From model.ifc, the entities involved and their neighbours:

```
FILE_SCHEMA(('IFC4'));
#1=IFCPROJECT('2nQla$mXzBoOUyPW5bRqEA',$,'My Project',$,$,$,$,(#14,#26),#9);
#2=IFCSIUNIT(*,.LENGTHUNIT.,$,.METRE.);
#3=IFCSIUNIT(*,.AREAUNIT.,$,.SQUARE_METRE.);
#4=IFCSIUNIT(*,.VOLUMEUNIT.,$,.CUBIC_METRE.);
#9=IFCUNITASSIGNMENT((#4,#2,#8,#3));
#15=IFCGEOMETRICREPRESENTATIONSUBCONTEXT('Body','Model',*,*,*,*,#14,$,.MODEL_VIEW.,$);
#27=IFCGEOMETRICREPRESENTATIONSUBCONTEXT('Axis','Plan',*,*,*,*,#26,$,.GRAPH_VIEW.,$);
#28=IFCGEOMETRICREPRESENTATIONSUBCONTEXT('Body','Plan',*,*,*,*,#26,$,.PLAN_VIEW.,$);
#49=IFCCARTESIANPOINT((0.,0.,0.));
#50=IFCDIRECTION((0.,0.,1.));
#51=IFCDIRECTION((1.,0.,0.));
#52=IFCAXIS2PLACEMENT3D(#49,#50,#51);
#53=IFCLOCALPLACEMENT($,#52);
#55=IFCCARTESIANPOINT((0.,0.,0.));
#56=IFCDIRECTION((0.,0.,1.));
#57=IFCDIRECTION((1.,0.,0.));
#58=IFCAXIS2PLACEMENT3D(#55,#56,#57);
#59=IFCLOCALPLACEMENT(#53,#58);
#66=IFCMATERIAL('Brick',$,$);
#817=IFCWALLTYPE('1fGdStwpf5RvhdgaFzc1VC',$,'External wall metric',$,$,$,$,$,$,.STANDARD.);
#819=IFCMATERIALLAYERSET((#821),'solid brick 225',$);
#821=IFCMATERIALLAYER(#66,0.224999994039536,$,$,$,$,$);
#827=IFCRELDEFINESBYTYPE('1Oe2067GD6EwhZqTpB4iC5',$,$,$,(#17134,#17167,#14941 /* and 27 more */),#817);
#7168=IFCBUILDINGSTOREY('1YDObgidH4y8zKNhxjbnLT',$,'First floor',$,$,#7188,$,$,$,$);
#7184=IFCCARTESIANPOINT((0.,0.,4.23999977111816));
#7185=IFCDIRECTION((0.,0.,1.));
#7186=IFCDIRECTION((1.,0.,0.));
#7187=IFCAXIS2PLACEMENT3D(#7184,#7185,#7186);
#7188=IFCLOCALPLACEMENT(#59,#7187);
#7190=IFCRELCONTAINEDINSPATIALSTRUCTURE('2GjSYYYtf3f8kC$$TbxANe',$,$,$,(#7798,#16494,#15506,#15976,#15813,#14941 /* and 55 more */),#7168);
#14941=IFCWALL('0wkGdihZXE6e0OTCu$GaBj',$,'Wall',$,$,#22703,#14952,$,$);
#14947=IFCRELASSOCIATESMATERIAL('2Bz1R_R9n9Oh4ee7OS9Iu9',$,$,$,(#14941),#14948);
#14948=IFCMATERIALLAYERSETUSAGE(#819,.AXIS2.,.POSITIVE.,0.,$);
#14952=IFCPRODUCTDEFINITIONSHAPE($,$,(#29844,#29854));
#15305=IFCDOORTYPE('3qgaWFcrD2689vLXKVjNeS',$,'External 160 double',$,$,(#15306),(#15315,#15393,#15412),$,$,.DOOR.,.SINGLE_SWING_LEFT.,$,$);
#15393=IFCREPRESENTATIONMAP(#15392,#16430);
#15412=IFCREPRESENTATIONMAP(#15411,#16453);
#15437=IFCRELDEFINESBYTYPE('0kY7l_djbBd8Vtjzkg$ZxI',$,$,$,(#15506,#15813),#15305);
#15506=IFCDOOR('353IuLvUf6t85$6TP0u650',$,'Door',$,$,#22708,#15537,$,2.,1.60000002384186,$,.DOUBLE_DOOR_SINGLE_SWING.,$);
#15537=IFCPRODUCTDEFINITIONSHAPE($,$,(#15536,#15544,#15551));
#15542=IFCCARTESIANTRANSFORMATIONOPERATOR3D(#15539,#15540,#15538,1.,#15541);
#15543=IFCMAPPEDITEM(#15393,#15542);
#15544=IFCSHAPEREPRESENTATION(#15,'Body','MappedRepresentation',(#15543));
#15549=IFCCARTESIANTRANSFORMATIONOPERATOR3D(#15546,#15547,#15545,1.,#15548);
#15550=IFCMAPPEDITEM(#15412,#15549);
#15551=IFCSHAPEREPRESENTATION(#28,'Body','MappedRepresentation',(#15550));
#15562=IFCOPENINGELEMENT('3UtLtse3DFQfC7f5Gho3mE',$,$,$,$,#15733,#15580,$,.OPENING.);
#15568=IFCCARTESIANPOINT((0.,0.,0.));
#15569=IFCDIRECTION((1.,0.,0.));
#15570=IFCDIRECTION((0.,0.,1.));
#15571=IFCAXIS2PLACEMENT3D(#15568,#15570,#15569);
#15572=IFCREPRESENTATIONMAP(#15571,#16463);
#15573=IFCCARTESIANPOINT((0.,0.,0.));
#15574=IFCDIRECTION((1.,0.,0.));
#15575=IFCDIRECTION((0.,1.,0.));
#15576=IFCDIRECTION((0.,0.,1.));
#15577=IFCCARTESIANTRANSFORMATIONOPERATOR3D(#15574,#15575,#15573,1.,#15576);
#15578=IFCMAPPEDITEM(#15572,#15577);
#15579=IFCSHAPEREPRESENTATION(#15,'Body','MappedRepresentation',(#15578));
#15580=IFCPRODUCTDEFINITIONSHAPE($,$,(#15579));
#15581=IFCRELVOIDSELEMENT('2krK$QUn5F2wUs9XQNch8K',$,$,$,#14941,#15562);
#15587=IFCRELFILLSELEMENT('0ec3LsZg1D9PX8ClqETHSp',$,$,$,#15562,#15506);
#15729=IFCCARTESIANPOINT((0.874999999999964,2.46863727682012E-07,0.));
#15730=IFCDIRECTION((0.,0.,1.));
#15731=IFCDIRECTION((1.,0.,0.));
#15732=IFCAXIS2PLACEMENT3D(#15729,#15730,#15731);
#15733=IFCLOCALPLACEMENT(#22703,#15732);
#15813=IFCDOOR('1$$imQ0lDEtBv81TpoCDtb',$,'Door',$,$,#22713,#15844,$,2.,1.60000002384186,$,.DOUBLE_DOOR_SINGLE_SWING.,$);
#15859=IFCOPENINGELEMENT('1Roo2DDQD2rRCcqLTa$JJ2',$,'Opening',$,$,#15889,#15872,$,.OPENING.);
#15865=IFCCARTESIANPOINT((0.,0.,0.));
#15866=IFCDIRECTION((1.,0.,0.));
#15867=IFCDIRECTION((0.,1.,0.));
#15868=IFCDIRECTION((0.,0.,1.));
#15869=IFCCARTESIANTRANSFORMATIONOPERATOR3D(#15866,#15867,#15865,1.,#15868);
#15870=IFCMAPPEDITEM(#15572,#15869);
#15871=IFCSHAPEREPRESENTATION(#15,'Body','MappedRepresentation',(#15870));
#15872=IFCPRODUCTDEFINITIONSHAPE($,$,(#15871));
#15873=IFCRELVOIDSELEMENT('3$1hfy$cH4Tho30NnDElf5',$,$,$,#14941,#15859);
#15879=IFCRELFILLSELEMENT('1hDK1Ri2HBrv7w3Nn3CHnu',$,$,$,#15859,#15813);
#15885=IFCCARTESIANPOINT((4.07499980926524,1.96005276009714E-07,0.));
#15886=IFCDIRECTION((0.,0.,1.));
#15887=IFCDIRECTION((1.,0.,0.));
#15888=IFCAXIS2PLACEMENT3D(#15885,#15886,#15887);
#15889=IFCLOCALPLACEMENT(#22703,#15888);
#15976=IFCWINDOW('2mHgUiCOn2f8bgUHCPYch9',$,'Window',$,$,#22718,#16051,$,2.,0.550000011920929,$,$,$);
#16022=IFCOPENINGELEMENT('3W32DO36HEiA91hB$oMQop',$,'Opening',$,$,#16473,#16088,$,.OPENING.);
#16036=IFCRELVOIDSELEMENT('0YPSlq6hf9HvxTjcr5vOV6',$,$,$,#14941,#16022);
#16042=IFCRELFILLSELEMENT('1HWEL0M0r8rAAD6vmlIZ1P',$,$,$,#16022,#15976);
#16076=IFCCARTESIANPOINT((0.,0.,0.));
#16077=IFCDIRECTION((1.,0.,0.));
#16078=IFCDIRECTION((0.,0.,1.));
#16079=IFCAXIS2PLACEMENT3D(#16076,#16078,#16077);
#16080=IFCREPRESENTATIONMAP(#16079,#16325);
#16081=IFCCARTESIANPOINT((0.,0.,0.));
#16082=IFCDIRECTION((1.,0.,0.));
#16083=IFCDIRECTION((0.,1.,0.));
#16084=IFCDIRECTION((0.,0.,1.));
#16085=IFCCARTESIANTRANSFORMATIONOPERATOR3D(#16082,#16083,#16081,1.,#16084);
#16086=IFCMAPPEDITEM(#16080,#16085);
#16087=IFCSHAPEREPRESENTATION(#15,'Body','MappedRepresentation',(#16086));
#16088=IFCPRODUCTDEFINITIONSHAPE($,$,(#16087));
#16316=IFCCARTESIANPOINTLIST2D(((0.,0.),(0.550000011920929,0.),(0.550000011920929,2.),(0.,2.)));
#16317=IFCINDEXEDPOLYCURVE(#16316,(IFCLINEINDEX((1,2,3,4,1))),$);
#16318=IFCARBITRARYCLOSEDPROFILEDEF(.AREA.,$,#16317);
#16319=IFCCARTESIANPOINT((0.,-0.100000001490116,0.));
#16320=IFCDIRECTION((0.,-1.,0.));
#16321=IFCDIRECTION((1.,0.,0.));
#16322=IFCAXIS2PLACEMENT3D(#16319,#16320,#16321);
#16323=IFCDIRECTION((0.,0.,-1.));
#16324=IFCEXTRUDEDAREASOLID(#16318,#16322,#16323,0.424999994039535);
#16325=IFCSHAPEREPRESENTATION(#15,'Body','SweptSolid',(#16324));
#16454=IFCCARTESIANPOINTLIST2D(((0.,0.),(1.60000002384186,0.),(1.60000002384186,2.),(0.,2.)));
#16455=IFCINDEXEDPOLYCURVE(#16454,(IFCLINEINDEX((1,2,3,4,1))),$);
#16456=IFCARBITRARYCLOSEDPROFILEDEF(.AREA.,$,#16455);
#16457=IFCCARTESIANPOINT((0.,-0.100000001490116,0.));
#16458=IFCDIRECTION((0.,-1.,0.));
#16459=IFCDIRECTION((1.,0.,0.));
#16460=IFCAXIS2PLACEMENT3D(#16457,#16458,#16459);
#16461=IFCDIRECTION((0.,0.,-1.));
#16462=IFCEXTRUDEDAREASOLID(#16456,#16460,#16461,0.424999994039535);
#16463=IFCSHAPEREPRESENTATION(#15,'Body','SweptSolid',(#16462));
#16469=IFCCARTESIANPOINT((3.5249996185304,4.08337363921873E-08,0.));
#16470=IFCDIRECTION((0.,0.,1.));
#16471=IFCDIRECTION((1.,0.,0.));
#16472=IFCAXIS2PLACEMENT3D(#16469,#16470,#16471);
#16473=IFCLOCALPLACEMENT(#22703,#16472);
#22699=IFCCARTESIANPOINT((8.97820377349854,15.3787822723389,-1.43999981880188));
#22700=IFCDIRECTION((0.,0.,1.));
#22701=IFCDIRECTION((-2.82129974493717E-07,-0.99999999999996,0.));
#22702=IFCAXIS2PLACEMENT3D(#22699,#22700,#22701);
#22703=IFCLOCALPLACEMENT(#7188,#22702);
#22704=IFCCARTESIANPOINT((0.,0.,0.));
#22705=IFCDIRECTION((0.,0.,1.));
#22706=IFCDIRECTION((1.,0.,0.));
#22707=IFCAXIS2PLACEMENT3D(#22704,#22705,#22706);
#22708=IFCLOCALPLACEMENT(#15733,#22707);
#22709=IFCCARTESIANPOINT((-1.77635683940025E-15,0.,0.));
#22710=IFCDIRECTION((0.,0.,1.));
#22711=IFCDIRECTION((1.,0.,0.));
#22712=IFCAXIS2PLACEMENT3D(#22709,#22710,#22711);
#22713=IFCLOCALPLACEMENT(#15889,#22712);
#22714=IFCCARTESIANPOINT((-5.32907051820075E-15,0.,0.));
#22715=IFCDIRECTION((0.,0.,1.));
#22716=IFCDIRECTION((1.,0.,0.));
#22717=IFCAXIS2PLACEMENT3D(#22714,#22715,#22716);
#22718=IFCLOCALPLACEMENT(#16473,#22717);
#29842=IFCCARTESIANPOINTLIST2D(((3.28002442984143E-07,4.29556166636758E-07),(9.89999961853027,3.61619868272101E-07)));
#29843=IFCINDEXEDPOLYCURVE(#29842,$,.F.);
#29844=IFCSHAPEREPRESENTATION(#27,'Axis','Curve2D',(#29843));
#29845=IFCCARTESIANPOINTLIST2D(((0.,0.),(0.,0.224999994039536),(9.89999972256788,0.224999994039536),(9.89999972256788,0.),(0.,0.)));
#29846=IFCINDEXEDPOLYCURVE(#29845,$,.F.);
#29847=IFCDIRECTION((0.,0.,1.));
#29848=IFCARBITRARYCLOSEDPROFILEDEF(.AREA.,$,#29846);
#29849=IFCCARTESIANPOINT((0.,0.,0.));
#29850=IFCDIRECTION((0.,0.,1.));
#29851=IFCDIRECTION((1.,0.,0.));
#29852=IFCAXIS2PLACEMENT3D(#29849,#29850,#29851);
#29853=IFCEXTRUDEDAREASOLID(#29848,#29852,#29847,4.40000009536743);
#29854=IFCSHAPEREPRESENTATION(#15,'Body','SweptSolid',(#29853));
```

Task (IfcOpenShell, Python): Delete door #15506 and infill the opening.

```python
import ifcopenshell
import ifcopenshell.api.feature
import ifcopenshell.api.root
import ifcopenshell.geom
import ifcopenshell.util.shape

model = ifcopenshell.open("model.ifc")
settings = ifcopenshell.geom.settings()


def volume(element):
    """Net volume in cubic metres, openings subtracted."""
    shape = ifcopenshell.geom.create_shape(settings, element)
    return ifcopenshell.util.shape.get_volume(shape.geometry)


door = model.by_guid("353IuLvUf6t85$6TP0u650")
opening = door.FillsVoids[0].RelatingOpeningElement
wall = opening.VoidsElements[0].RelatingBuildingElement
before = volume(wall)

ifcopenshell.api.root.remove_product(model, product=door)
ifcopenshell.api.feature.remove_feature(model, feature=opening)

after = volume(wall)

print(f"wall volume {before:.3f} -> {after:.3f} m3")

model.write("model_updated.ifc")
```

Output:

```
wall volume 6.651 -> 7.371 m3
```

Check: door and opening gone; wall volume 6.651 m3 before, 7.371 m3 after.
